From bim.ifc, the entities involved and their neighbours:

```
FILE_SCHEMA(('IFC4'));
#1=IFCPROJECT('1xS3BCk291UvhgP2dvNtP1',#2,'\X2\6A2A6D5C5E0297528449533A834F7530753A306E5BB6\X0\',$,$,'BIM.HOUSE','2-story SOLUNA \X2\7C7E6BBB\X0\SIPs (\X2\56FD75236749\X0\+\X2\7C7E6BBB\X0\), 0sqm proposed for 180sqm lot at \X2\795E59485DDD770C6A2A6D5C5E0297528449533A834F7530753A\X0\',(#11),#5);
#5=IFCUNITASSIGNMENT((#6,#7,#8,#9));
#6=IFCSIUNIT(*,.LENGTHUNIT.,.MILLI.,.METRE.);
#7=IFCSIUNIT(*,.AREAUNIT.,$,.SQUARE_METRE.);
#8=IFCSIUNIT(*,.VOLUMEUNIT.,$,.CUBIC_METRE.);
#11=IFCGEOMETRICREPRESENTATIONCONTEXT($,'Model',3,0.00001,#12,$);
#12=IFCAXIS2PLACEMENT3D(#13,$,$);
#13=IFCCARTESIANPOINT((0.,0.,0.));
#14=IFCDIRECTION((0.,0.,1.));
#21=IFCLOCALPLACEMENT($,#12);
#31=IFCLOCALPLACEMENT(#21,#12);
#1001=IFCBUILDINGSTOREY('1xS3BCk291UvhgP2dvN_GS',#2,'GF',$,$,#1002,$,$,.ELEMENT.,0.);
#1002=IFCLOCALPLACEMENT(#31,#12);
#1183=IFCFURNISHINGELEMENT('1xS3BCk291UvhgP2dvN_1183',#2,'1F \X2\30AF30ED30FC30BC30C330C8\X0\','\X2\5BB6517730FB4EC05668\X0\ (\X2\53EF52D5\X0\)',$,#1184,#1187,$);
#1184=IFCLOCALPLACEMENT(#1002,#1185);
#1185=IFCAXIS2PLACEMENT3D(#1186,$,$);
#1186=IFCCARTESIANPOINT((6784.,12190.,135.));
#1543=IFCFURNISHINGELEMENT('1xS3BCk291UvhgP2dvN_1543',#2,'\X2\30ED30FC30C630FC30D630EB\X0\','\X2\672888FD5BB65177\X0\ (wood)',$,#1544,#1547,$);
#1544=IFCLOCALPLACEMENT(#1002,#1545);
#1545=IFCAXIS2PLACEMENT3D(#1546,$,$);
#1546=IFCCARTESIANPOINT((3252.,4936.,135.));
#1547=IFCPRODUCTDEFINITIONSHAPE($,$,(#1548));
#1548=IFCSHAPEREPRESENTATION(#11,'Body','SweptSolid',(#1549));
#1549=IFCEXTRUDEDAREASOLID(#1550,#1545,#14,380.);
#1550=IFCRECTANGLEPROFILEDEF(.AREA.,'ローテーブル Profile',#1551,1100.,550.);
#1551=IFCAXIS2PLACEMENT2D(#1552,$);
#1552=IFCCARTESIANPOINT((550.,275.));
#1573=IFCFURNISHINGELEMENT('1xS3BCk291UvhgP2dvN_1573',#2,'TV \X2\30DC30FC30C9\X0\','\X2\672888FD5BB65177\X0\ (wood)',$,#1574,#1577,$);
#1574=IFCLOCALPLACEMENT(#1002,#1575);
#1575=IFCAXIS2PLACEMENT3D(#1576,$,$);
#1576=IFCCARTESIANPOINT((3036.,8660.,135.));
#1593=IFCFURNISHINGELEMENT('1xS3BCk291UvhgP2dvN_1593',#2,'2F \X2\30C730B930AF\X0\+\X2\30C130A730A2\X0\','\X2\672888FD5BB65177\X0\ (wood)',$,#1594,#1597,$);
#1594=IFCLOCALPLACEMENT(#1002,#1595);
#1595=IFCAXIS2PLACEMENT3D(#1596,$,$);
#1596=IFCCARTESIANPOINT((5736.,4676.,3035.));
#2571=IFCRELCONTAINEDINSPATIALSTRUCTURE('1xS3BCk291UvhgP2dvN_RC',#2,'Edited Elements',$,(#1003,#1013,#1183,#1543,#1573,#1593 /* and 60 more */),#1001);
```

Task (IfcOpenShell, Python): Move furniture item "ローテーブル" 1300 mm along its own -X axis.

```python
import ifcopenshell
import ifcopenshell.api.geometry
import ifcopenshell.util.placement
import ifcopenshell.util.unit

model = ifcopenshell.open("bim.ifc")
unit_scale = ifcopenshell.util.unit.calculate_unit_scale(model)

item = model.by_guid("1xS3BCk291UvhgP2dvN_1543")
matrix = ifcopenshell.util.placement.get_local_placement(item.ObjectPlacement)
matrix[:3, 3] -= matrix[:3, 0] * 1.3 / unit_scale
ifcopenshell.api.geometry.edit_object_placement(model, product=item, matrix=matrix, is_si=False)

print(ifcopenshell.util.placement.get_local_placement(item.ObjectPlacement).round(3) + 0.0)

model.write("bim_v2.ifc")
```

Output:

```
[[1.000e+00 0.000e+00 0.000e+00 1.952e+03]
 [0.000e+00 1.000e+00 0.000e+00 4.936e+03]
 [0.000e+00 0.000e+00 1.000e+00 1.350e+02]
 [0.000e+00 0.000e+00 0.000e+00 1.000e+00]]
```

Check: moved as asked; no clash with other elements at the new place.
